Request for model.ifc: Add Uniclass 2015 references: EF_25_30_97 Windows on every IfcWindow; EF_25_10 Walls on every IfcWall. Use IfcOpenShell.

First a look at what the model holds.

```python
import ifcopenshell

model = ifcopenshell.open("model.ifc")
print(model.schema)
print("classifications:", [c.Name for c in model.by_type("IfcClassification")])
for ifc_class in ("IfcDoor", "IfcRoof", "IfcStair", "IfcWall", "IfcWindow"):
    print(ifc_class, len(model.by_type(ifc_class)))
```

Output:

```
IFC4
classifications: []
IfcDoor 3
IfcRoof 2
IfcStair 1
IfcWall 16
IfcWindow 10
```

```python
import ifcopenshell
import ifcopenshell.api.classification

model = ifcopenshell.open("model.ifc")

system = ifcopenshell.api.classification.add_classification(model, classification="Uniclass 2015")

codes = {
    "IfcWindow": ("EF_25_30_97", "Windows"),
    "IfcWall": ("EF_25_10", "Walls"),
}
for ifc_class, (code, name) in codes.items():
    products = model.by_type(ifc_class)
    ifcopenshell.api.classification.add_reference(
        model, products=products, classification=system, identification=code, name=name
    )
    print(code, len(products))

model.write("model_rev.ifc")
```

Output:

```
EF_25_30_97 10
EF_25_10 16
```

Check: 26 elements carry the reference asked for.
